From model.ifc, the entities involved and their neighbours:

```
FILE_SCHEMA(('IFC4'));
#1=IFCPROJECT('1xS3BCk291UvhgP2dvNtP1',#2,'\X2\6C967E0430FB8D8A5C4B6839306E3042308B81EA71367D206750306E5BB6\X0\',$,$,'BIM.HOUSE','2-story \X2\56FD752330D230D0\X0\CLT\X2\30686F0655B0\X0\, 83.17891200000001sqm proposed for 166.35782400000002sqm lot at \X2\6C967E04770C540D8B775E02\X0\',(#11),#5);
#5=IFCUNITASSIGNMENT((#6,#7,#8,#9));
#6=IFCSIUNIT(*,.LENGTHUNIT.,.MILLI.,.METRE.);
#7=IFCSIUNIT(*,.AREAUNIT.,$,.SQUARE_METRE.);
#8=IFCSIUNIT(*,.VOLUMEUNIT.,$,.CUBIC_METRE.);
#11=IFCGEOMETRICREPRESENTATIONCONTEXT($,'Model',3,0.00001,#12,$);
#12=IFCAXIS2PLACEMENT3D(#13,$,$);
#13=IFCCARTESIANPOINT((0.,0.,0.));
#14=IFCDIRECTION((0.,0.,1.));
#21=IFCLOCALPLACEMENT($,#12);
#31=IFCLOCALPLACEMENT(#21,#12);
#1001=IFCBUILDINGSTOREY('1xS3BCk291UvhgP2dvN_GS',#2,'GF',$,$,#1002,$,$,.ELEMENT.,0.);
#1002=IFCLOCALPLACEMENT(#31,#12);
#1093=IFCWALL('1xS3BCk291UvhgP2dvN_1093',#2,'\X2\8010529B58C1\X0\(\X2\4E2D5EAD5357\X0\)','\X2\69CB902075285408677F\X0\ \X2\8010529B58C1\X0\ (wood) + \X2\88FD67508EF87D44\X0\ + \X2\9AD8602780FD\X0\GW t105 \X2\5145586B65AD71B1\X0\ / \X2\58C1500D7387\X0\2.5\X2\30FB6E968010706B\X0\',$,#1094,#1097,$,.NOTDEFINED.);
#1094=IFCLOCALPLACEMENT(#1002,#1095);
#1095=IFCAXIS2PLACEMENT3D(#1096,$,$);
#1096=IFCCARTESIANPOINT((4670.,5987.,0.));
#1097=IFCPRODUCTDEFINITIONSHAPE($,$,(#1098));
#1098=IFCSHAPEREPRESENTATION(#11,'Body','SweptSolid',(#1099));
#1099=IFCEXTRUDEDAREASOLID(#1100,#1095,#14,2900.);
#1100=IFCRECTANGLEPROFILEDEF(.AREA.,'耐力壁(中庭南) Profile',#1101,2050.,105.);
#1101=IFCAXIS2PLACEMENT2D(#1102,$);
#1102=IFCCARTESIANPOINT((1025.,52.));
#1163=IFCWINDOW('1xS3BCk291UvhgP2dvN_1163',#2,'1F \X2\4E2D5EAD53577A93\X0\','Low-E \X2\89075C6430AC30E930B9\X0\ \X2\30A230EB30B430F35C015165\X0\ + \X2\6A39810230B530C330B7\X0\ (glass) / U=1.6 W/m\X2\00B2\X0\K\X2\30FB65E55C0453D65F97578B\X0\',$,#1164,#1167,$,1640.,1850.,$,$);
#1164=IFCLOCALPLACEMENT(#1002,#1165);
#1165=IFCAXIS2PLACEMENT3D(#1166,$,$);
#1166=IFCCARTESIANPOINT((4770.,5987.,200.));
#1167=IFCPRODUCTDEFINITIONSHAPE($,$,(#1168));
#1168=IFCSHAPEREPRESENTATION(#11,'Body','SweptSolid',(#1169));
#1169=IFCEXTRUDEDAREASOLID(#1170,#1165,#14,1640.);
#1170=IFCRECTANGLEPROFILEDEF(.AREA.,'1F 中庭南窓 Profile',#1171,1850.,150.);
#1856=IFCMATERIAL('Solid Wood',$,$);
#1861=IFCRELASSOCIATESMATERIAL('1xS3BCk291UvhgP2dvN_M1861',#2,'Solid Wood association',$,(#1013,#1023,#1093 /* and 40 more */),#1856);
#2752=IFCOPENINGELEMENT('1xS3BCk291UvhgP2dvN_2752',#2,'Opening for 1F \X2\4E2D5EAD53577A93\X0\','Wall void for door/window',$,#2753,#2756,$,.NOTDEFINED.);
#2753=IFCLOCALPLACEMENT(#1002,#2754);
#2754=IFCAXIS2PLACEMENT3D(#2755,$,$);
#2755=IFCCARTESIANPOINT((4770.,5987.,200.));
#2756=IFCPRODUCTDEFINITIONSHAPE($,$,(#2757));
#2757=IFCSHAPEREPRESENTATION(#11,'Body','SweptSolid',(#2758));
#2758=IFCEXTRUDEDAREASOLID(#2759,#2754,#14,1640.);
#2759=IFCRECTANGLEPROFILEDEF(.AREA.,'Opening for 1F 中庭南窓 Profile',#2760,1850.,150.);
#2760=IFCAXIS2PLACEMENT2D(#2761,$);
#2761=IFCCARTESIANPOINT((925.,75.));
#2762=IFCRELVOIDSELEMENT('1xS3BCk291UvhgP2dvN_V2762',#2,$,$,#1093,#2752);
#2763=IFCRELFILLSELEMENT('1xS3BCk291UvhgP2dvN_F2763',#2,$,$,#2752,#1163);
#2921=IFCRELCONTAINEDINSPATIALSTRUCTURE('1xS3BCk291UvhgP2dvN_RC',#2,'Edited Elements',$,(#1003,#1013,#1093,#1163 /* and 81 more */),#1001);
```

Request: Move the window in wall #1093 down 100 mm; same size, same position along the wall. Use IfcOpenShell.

```python
import numpy as np
import ifcopenshell
import ifcopenshell.api.geometry
import ifcopenshell.util.placement
import ifcopenshell.util.unit

model = ifcopenshell.open("model.ifc")
unit_scale = ifcopenshell.util.unit.calculate_unit_scale(model)

window = model.by_guid("1xS3BCk291UvhgP2dvN_1163")
opening = window.FillsVoids[0].RelatingOpeningElement
dz = -100.0

shift = np.array([0.0, 0.0, dz])
# The window is not placed relative to its opening, so move both.
for product in (opening, window):
    matrix = ifcopenshell.util.placement.get_local_placement(product.ObjectPlacement)
    matrix[:3, 3] += shift
    ifcopenshell.api.geometry.edit_object_placement(model, product=product, matrix=matrix, is_si=False)

print(f"moved by {dz * unit_scale:+.3f} m")

model.write("model_updated.ifc")
```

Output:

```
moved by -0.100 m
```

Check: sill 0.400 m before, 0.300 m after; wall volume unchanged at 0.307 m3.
